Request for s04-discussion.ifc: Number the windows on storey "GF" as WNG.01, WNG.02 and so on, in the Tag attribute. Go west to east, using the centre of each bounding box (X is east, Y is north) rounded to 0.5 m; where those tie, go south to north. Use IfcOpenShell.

First a look at what the model holds.

```python
import ifcopenshell
import ifcopenshell.util.element
import ifcopenshell.util.placement

model = ifcopenshell.open("s04-discussion.ifc")
print(model.schema)
storey = next(s for s in model.by_type("IfcBuildingStorey") if s.Name == "GF")
windows = [e for e in ifcopenshell.util.element.get_decomposition(storey) if e.is_a("IfcWindow")]
for e in sorted(windows, key=lambda e: e.id()):
    origin = ifcopenshell.util.placement.get_local_placement(e.ObjectPlacement)[:3, 3]
    print(e.id(), e.Tag, e.Name, origin.round(2) + 0.0, sep=" | ")
```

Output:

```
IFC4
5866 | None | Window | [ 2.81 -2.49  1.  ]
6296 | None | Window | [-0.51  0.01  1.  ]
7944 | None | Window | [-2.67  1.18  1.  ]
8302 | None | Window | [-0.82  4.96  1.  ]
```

```python
import ifcopenshell
import ifcopenshell.geom
import ifcopenshell.util.element
import ifcopenshell.util.shape

model = ifcopenshell.open("s04-discussion.ifc")
settings = ifcopenshell.geom.settings()
settings.set("use-world-coords", True)


def centre(element):
    shape = ifcopenshell.geom.create_shape(settings, element)
    return ifcopenshell.util.shape.get_bbox_centroid(shape.geometry)


storey = next(s for s in model.by_type("IfcBuildingStorey") if s.Name == "GF")
windows = [e for e in ifcopenshell.util.element.get_decomposition(storey) if e.is_a("IfcWindow")]

# Insertion points can sit at a corner or the storey origin, so sort by the geometry (in metres).
centres = {e: centre(e) for e in windows}
windows.sort(key=lambda e: (round(centres[e][0] / 0.5), centres[e][1]))

for i, e in enumerate(windows, start=1):
    number = f"WNG.{i:02d}"
    e.Tag = number
    print(e.id(), number)

model.write("s04-discussion-out.ifc")
```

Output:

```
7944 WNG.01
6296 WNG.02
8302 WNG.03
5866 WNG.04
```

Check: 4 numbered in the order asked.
